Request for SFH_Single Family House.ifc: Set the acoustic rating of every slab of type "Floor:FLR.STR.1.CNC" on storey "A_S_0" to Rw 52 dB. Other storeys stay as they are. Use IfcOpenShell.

First a look at what the model holds.

```python
import ifcopenshell
import ifcopenshell.util.element

model = ifcopenshell.open("SFH_Single Family House.ifc")
print(model.schema)
storey = next(s for s in model.by_type("IfcBuildingStorey") if s.Name == "A_S_0")
slabs = [e for e in ifcopenshell.util.element.get_decomposition(storey) if e.is_a("IfcSlab")]
seen = {}
for e in slabs:
    element_type = ifcopenshell.util.element.get_type(e)
    key = (element_type.Name if element_type != e and element_type else None, ifcopenshell.util.element.get_pset(e, "Pset_SlabCommon", "AcousticRating"))
    seen[key] = seen.get(key, 0) + 1
for (name, value), count in sorted(seen.items(), key=str):
    print(count, "x", name, "|", value)
```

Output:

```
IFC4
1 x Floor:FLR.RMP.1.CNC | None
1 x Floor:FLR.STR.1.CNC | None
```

```python
import ifcopenshell
import ifcopenshell.api.pset
import ifcopenshell.util.element

model = ifcopenshell.open("SFH_Single Family House.ifc")

storey = next(s for s in model.by_type("IfcBuildingStorey") if s.Name == "A_S_0")
slabs = [e for e in ifcopenshell.util.element.get_decomposition(storey) if e.is_a("IfcSlab")]

count = 0
for e in slabs:
    element_type = ifcopenshell.util.element.get_type(e)
    if element_type in (None, e) or element_type.Name != "Floor:FLR.STR.1.CNC":
        continue
    # add_pset returns the element's existing set when there is one.
    pset = ifcopenshell.api.pset.add_pset(model, product=e, name="Pset_SlabCommon")
    ifcopenshell.api.pset.edit_pset(model, pset=pset, properties={"AcousticRating": "Rw 52 dB"})
    count += 1

print(count, "slabs updated")

model.write("SFH_Single Family House-out.ifc")
```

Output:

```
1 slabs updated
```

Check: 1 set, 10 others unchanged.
